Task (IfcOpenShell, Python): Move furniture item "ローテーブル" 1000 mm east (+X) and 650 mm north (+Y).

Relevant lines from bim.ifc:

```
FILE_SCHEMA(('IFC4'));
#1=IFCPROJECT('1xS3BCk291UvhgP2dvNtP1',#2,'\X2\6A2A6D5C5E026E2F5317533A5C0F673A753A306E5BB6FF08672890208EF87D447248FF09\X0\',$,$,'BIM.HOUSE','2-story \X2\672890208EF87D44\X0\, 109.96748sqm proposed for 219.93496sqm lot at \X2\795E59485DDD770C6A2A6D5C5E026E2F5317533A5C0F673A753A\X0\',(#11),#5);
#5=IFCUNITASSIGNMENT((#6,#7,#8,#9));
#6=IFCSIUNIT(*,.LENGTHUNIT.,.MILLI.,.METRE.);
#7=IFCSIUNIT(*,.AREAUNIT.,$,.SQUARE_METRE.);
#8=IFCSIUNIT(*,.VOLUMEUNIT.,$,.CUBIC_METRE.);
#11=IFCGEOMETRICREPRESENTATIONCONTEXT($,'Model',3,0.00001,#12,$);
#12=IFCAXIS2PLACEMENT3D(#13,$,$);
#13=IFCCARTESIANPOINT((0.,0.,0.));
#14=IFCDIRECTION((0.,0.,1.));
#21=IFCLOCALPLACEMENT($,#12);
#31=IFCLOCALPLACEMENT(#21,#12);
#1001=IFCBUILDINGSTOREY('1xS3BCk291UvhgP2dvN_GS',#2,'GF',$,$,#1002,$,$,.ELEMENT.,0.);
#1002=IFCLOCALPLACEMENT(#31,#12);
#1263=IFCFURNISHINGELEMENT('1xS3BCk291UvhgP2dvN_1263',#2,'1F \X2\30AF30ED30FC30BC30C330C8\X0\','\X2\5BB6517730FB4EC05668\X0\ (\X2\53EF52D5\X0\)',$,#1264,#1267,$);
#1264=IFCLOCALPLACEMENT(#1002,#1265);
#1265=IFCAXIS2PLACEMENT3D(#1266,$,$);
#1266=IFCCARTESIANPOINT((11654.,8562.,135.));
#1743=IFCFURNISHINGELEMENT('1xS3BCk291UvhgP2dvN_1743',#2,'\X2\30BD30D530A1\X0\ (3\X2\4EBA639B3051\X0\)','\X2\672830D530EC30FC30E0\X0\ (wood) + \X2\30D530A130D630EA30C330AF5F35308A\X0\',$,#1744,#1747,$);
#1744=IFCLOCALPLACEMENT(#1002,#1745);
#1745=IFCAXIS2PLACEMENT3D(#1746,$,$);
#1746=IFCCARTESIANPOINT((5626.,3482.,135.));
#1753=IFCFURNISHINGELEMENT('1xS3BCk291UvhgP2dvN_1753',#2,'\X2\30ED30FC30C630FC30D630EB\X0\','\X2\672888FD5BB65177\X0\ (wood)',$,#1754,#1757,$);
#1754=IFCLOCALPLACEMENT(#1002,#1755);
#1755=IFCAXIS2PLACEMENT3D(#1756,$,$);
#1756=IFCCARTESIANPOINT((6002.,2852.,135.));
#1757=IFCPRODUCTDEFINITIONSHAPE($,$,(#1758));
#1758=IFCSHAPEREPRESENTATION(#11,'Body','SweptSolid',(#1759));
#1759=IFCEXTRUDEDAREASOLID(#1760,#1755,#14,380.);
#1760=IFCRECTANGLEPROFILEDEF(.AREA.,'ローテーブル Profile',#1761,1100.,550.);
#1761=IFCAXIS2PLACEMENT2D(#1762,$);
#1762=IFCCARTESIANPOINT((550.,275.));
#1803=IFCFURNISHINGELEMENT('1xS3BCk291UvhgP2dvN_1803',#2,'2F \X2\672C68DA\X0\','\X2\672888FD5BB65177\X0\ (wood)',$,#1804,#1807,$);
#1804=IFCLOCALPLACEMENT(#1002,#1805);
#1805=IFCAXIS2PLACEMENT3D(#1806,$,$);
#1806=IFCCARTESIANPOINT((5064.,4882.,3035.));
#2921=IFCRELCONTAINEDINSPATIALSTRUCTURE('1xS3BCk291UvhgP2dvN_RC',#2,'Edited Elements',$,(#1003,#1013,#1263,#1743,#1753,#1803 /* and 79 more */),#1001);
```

```python
import ifcopenshell
import ifcopenshell.api.geometry
import ifcopenshell.util.placement
import ifcopenshell.util.unit

model = ifcopenshell.open("bim.ifc")
unit_scale = ifcopenshell.util.unit.calculate_unit_scale(model)

item = model.by_id(1753)
matrix = ifcopenshell.util.placement.get_local_placement(item.ObjectPlacement)
matrix[0, 3] += 1 / unit_scale
matrix[1, 3] += 0.65 / unit_scale
ifcopenshell.api.geometry.edit_object_placement(model, product=item, matrix=matrix, is_si=False)

print(ifcopenshell.util.placement.get_local_placement(item.ObjectPlacement).round(3) + 0.0)

model.write("bim_rev.ifc")
```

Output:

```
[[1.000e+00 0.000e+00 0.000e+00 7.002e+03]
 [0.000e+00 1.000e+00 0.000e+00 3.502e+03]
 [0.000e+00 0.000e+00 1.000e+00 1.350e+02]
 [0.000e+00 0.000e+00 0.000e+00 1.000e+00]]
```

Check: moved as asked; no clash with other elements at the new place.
